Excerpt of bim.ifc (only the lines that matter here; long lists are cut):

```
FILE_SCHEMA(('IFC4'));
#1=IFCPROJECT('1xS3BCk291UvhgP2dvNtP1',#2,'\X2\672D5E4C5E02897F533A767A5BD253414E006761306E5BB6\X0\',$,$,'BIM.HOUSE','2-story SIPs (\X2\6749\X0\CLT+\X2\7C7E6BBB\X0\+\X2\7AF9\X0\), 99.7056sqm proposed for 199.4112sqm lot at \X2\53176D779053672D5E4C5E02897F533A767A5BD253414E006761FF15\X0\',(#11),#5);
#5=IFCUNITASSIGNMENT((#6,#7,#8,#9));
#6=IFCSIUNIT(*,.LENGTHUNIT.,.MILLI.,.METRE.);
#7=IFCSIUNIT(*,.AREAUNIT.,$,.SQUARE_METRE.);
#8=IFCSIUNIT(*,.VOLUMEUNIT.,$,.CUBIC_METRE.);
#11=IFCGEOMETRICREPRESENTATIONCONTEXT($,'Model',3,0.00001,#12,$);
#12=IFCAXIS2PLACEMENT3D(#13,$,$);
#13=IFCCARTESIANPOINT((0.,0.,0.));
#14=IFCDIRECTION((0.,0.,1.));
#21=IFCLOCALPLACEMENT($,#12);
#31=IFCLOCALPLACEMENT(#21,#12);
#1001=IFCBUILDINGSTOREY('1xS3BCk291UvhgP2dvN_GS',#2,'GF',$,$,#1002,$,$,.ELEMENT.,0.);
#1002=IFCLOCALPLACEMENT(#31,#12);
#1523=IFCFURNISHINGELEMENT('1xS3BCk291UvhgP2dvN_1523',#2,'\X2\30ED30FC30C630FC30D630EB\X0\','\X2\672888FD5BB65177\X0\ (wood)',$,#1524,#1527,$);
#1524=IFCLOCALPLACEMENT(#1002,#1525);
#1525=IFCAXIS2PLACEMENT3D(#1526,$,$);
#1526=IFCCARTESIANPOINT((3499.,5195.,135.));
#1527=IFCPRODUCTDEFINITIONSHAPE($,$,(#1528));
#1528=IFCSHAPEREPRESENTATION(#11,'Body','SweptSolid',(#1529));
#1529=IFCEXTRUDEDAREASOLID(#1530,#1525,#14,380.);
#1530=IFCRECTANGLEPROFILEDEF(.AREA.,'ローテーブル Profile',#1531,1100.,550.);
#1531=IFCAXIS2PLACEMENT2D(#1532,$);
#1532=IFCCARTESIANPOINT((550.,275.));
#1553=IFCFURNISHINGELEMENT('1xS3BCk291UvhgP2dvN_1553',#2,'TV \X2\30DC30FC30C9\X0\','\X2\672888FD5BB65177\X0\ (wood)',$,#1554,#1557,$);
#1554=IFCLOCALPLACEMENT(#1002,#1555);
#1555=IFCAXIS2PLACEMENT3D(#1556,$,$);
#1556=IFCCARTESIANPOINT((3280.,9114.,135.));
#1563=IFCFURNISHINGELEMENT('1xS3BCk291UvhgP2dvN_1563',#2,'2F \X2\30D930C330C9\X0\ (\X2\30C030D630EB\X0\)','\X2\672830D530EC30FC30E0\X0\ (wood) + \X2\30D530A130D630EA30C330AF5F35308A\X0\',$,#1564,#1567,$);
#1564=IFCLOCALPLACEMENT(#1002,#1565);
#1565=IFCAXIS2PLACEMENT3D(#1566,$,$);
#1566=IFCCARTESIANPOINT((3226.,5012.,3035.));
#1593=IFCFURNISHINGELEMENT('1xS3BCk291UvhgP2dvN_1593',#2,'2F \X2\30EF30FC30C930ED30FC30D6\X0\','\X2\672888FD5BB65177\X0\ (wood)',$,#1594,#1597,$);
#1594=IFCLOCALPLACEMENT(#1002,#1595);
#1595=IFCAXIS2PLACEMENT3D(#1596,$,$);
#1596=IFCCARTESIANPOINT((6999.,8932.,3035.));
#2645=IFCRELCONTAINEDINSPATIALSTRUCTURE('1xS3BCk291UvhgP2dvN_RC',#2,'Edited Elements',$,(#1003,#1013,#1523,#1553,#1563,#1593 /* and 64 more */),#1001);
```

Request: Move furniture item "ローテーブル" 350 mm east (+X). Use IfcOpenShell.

```python
import ifcopenshell
import ifcopenshell.api.geometry
import ifcopenshell.util.placement
import ifcopenshell.util.unit

model = ifcopenshell.open("bim.ifc")
unit_scale = ifcopenshell.util.unit.calculate_unit_scale(model)

item = model.by_guid("1xS3BCk291UvhgP2dvN_1523")
matrix = ifcopenshell.util.placement.get_local_placement(item.ObjectPlacement)
matrix[0, 3] += 0.35 / unit_scale
ifcopenshell.api.geometry.edit_object_placement(model, product=item, matrix=matrix, is_si=False)

print(ifcopenshell.util.placement.get_local_placement(item.ObjectPlacement).round(3) + 0.0)

model.write("bim_updated.ifc")
```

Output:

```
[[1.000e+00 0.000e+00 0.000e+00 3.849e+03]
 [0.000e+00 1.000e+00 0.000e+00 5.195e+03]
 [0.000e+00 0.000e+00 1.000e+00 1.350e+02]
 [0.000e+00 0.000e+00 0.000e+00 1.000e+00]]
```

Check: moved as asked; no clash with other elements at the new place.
